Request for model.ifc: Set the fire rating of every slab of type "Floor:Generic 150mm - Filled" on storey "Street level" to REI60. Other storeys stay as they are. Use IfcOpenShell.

First a look at what the model holds.

```python
import ifcopenshell
import ifcopenshell.util.element

model = ifcopenshell.open("model.ifc")
print(model.schema)
storey = next(s for s in model.by_type("IfcBuildingStorey") if s.Name == "Street level")
slabs = [e for e in ifcopenshell.util.element.get_decomposition(storey) if e.is_a("IfcSlab")]
seen = {}
for e in slabs:
    element_type = ifcopenshell.util.element.get_type(e)
    key = (element_type.Name if element_type != e and element_type else None, ifcopenshell.util.element.get_pset(e, "Pset_SlabCommon", "FireRating"))
    seen[key] = seen.get(key, 0) + 1
for (name, value), count in sorted(seen.items(), key=str):
    print(count, "x", name, "|", value)
```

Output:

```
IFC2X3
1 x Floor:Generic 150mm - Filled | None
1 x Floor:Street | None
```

```python
import ifcopenshell
import ifcopenshell.api.pset
import ifcopenshell.util.element

model = ifcopenshell.open("model.ifc")

storey = next(s for s in model.by_type("IfcBuildingStorey") if s.Name == "Street level")
slabs = [e for e in ifcopenshell.util.element.get_decomposition(storey) if e.is_a("IfcSlab")]

count = 0
for e in slabs:
    element_type = ifcopenshell.util.element.get_type(e)
    if element_type in (None, e) or element_type.Name != "Floor:Generic 150mm - Filled":
        continue
    # add_pset returns the element's existing set when there is one.
    pset = ifcopenshell.api.pset.add_pset(model, product=e, name="Pset_SlabCommon")
    ifcopenshell.api.pset.edit_pset(model, pset=pset, properties={"FireRating": "REI60"})
    count += 1

print(count, "slabs updated")

model.write("model_edited.ifc")
```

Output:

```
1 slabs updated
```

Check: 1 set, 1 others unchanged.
